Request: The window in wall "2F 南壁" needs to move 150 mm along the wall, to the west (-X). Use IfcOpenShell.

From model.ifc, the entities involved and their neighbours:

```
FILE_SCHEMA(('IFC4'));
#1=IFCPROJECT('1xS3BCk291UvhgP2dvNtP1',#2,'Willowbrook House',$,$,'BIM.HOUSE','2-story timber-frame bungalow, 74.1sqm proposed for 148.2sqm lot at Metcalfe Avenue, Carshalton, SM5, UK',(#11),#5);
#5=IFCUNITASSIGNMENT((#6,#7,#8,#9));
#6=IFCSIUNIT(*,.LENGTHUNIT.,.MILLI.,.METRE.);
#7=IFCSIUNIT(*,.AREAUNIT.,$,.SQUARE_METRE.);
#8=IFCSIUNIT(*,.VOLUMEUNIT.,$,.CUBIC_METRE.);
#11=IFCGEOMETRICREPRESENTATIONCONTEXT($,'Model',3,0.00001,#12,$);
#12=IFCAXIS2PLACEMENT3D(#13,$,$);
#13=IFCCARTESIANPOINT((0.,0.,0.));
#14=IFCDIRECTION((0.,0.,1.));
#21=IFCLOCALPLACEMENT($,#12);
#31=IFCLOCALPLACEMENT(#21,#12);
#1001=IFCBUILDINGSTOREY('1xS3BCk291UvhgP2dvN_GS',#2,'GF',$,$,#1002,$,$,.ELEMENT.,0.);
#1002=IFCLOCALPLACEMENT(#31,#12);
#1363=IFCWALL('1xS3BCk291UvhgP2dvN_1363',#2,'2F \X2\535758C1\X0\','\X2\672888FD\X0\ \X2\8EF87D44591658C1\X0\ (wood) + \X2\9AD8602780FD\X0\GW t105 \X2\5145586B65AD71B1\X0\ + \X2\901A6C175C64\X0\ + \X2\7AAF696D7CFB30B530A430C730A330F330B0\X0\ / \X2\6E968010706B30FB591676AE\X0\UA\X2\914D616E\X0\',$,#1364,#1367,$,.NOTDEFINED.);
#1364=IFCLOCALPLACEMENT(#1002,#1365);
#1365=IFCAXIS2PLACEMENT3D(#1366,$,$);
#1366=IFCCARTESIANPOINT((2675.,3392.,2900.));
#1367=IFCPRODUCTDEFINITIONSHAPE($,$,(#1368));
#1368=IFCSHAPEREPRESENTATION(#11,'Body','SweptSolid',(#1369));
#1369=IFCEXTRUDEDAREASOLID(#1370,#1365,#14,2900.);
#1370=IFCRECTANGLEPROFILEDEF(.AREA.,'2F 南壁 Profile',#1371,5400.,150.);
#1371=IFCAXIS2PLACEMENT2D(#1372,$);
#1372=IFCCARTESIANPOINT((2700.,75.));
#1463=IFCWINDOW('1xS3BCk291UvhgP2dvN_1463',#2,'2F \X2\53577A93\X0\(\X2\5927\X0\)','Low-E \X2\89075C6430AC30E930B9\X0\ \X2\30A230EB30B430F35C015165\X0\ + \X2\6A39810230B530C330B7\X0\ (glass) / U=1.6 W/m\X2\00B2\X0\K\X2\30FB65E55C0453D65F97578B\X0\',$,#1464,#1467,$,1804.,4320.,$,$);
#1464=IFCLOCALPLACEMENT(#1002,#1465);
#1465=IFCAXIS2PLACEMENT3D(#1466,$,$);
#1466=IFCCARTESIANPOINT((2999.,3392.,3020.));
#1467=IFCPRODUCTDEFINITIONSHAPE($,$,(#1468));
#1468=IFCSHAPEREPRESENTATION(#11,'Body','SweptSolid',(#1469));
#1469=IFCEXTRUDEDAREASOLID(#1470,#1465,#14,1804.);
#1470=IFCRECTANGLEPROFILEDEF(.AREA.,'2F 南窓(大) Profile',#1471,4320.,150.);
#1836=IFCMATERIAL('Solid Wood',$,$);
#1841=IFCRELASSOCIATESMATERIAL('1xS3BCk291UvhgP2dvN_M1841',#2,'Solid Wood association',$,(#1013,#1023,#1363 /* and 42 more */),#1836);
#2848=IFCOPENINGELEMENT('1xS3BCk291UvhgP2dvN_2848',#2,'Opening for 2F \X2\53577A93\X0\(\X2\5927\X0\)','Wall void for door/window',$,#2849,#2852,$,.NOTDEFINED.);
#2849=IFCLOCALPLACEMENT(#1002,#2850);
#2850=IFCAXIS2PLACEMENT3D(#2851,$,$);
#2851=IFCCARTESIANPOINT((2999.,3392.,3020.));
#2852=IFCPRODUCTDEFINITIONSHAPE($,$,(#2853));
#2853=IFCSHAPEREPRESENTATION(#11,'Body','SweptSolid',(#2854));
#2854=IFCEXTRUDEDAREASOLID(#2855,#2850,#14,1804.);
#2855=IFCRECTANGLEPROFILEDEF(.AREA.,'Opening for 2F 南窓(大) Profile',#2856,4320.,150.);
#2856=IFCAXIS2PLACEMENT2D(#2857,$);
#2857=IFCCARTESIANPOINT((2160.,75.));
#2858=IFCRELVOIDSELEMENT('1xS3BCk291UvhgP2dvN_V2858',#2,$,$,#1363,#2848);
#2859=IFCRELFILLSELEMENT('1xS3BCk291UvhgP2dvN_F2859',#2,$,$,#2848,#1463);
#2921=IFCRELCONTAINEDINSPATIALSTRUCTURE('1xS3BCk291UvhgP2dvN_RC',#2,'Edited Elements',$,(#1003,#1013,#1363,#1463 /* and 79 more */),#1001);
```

```python
import ifcopenshell
import ifcopenshell.api.geometry
import ifcopenshell.util.placement
import ifcopenshell.util.unit

model = ifcopenshell.open("model.ifc")
unit_scale = ifcopenshell.util.unit.calculate_unit_scale(model)

window = model.by_guid("1xS3BCk291UvhgP2dvN_1463")
opening = window.FillsVoids[0].RelatingOpeningElement
wall = opening.VoidsElements[0].RelatingBuildingElement

wall_matrix = ifcopenshell.util.placement.get_local_placement(wall.ObjectPlacement)
shift = wall_matrix[:3, 0] * -0.15 / unit_scale
before = ifcopenshell.util.placement.get_local_placement(window.ObjectPlacement)[:3, 3].copy()

# The window is not placed relative to its opening, so move both.
for product in (opening, window):
    matrix = ifcopenshell.util.placement.get_local_placement(product.ObjectPlacement)
    matrix[:3, 3] += shift
    ifcopenshell.api.geometry.edit_object_placement(model, product=product, matrix=matrix, is_si=False)

after = ifcopenshell.util.placement.get_local_placement(window.ObjectPlacement)[:3, 3]
print("window moved by", (after - before).round(3) + 0.0)

model.write("model_edited.ifc")
```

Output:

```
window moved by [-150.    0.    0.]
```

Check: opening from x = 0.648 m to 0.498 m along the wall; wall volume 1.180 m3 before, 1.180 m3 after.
